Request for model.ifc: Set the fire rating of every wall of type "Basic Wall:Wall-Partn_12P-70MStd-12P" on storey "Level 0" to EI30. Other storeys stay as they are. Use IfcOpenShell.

First a look at what the model holds.

```python
import ifcopenshell
import ifcopenshell.util.element

model = ifcopenshell.open("model.ifc")
print(model.schema)
storey = next(s for s in model.by_type("IfcBuildingStorey") if s.Name == "Level 0")
walls = [e for e in ifcopenshell.util.element.get_decomposition(storey) if e.is_a("IfcWall")]
seen = {}
for e in walls:
    element_type = ifcopenshell.util.element.get_type(e)
    key = (element_type.Name if element_type != e and element_type else None, ifcopenshell.util.element.get_pset(e, "Pset_WallCommon", "FireRating"))
    seen[key] = seen.get(key, 0) + 1
for (name, value), count in sorted(seen.items(), key=str):
    print(count, "x", name, "|", value)
```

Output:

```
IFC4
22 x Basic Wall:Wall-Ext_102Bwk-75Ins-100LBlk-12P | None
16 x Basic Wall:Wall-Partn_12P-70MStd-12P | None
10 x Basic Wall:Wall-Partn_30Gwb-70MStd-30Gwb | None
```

```python
import ifcopenshell
import ifcopenshell.api.pset
import ifcopenshell.util.element

model = ifcopenshell.open("model.ifc")

storey = next(s for s in model.by_type("IfcBuildingStorey") if s.Name == "Level 0")
walls = [e for e in ifcopenshell.util.element.get_decomposition(storey) if e.is_a("IfcWall")]

count = 0
for e in walls:
    element_type = ifcopenshell.util.element.get_type(e)
    if element_type in (None, e) or element_type.Name != "Basic Wall:Wall-Partn_12P-70MStd-12P":
        continue
    # add_pset returns the element's existing set when there is one.
    pset = ifcopenshell.api.pset.add_pset(model, product=e, name="Pset_WallCommon")
    ifcopenshell.api.pset.edit_pset(model, pset=pset, properties={"FireRating": "EI30"})
    count += 1

print(count, "walls updated")

model.write("model-out.ifc")
```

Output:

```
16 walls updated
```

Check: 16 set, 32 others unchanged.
